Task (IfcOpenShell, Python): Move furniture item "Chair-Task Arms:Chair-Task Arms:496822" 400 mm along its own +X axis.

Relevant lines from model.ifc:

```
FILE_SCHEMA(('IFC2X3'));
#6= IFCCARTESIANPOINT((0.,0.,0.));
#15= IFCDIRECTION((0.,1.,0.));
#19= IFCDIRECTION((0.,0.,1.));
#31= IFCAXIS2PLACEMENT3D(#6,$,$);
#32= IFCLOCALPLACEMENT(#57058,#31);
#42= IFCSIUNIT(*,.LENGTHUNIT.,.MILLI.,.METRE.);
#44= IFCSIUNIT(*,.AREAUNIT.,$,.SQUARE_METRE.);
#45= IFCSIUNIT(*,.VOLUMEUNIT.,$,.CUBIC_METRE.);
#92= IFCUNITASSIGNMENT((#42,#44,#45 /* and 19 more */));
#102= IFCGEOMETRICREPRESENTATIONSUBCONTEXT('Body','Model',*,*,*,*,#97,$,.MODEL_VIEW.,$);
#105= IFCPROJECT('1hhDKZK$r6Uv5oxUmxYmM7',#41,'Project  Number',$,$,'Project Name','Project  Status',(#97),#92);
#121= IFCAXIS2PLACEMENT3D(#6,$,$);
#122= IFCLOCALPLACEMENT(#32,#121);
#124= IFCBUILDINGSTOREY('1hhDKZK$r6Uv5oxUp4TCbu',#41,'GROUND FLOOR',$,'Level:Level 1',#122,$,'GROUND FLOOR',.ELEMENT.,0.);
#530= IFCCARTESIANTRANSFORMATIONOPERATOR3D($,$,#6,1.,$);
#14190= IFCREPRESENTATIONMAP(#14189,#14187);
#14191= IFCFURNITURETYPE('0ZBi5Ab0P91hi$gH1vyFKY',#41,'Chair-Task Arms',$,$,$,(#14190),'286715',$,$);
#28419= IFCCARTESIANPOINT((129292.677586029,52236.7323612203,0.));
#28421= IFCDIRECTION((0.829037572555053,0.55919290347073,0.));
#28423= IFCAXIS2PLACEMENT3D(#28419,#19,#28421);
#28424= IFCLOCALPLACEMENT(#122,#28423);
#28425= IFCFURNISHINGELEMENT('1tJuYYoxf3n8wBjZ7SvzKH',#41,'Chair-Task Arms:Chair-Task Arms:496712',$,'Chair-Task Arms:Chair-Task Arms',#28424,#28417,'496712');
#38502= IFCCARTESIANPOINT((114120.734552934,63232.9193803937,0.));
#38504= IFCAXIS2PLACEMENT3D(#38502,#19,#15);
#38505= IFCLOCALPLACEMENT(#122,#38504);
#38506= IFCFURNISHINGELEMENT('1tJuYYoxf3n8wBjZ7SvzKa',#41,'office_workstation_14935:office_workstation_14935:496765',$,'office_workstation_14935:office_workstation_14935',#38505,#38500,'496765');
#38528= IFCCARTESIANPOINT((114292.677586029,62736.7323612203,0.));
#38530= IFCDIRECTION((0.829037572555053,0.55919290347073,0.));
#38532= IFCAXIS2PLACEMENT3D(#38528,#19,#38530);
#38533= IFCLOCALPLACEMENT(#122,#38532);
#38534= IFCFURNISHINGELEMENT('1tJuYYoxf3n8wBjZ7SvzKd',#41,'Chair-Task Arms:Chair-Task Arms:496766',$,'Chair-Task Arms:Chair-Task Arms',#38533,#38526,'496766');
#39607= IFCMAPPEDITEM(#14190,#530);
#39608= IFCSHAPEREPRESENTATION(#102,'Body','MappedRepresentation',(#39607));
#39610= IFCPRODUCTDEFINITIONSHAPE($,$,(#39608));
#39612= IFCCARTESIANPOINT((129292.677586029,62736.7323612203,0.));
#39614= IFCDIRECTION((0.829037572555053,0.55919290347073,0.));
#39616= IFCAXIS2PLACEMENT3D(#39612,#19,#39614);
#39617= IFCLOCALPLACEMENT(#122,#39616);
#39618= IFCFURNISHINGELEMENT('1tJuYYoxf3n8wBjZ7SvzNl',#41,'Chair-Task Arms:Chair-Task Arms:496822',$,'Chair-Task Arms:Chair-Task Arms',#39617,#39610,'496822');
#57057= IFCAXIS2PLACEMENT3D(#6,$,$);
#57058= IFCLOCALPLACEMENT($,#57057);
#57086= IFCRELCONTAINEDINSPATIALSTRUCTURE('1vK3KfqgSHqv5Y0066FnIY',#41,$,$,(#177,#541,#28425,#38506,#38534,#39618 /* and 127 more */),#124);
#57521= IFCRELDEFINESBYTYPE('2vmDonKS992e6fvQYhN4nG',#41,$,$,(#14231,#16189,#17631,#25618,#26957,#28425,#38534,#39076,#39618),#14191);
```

```python
import ifcopenshell
import ifcopenshell.api.geometry
import ifcopenshell.util.placement
import ifcopenshell.util.unit

model = ifcopenshell.open("model.ifc")
unit_scale = ifcopenshell.util.unit.calculate_unit_scale(model)

item = model.by_guid("1tJuYYoxf3n8wBjZ7SvzNl")
matrix = ifcopenshell.util.placement.get_local_placement(item.ObjectPlacement)
matrix[:3, 3] += matrix[:3, 0] * 0.4 / unit_scale
ifcopenshell.api.geometry.edit_object_placement(model, product=item, matrix=matrix, is_si=False)

print(ifcopenshell.util.placement.get_local_placement(item.ObjectPlacement).round(3) + 0.0)

model.write("model_v2.ifc")
```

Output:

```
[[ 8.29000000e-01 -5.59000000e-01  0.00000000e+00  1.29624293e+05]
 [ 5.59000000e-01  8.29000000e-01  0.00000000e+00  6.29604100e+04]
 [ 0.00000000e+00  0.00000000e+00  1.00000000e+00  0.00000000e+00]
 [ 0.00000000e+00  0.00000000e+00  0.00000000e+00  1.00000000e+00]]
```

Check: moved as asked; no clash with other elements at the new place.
